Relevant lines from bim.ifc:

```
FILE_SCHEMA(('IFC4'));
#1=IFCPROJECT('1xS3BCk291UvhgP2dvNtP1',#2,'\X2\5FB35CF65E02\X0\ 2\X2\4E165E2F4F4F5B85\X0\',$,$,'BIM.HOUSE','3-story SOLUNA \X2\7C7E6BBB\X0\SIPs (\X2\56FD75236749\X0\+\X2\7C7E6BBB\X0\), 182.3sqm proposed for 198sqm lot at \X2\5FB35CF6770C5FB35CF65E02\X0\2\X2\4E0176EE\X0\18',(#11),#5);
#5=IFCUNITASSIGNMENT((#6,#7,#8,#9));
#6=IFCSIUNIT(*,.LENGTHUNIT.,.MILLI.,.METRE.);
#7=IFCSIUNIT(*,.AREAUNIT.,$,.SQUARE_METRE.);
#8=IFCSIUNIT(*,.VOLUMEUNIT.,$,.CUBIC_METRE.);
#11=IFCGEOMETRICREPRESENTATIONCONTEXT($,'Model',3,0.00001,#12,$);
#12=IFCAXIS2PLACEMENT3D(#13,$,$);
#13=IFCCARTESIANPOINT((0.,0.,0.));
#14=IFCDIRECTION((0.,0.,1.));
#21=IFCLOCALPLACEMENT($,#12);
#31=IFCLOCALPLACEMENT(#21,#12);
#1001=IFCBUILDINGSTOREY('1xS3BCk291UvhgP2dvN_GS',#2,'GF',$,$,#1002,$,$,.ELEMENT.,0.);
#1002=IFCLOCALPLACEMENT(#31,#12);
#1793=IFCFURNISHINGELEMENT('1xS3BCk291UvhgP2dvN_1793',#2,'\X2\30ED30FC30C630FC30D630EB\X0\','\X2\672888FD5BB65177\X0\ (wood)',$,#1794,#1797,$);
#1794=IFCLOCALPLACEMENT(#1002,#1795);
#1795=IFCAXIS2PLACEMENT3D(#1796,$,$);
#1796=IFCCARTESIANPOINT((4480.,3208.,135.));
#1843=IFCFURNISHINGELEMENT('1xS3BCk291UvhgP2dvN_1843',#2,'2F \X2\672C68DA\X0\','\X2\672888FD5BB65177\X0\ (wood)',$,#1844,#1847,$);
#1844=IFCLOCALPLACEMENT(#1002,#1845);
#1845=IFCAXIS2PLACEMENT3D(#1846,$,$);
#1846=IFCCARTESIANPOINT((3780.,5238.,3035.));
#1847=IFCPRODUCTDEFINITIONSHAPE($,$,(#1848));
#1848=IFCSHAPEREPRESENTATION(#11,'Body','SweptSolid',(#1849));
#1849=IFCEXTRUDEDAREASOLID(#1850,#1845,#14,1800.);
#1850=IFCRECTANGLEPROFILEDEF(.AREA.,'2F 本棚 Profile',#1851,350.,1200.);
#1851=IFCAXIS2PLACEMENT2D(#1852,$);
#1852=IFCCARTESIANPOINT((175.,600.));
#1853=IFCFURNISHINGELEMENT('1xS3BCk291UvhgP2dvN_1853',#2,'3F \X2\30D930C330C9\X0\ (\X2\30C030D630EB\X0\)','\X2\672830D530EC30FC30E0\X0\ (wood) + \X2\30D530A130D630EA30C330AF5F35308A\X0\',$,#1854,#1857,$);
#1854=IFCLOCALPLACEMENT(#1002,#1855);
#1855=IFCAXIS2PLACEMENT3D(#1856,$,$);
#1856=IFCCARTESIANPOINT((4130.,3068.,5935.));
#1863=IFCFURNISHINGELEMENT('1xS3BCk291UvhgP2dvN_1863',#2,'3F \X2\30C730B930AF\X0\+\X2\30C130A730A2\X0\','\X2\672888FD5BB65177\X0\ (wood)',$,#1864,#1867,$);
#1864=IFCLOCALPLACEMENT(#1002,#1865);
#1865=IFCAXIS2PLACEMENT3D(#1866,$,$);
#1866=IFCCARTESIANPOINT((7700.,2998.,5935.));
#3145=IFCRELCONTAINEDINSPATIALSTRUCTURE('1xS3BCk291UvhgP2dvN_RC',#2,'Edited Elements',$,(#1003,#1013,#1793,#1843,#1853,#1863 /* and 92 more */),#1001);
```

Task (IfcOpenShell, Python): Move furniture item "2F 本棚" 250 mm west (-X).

```python
import ifcopenshell
import ifcopenshell.api.geometry
import ifcopenshell.util.placement
import ifcopenshell.util.unit

model = ifcopenshell.open("bim.ifc")
unit_scale = ifcopenshell.util.unit.calculate_unit_scale(model)

item = model.by_guid("1xS3BCk291UvhgP2dvN_1843")
matrix = ifcopenshell.util.placement.get_local_placement(item.ObjectPlacement)
matrix[0, 3] -= 0.25 / unit_scale
ifcopenshell.api.geometry.edit_object_placement(model, product=item, matrix=matrix, is_si=False)

print(ifcopenshell.util.placement.get_local_placement(item.ObjectPlacement).round(3) + 0.0)

model.write("bim-out.ifc")
```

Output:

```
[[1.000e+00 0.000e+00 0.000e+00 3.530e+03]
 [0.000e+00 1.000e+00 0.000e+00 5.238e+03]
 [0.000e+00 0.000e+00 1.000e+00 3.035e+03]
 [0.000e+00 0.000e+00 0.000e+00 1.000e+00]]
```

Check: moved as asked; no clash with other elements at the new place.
